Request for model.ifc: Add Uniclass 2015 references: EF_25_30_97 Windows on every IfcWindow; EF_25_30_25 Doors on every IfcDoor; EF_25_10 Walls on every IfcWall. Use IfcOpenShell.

First a look at what the model holds.

```python
import ifcopenshell

model = ifcopenshell.open("model.ifc")
print(model.schema)
print("classifications:", [c.Name for c in model.by_type("IfcClassification")])
for ifc_class in ("IfcDoor", "IfcRoof", "IfcStair", "IfcWall", "IfcWindow"):
    print(ifc_class, len(model.by_type(ifc_class)))
```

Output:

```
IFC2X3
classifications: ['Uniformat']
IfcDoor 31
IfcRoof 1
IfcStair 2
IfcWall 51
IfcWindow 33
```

```python
import ifcopenshell
import ifcopenshell.api.classification

model = ifcopenshell.open("model.ifc")

# IFC2X3 requires Source and Edition and has no link from the project to the system.
system = model.create_entity("IfcClassification", Source="NBS", Edition="2015", Name="Uniclass 2015")

codes = {
    "IfcWindow": ("EF_25_30_97", "Windows"),
    "IfcDoor": ("EF_25_30_25", "Doors"),
    "IfcWall": ("EF_25_10", "Walls"),
}
for ifc_class, (code, name) in codes.items():
    products = model.by_type(ifc_class)
    ifcopenshell.api.classification.add_reference(
        model, products=products, classification=system, identification=code, name=name
    )
    print(code, len(products))

model.write("model-out.ifc")
```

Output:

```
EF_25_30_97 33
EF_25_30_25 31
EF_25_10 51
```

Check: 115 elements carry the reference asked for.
